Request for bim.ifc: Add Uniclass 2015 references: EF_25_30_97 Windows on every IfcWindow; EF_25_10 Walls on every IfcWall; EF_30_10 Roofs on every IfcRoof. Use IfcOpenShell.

First a look at what the model holds.

```python
import ifcopenshell

model = ifcopenshell.open("bim.ifc")
print(model.schema)
print("classifications:", [c.Name for c in model.by_type("IfcClassification")])
for ifc_class in ("IfcDoor", "IfcRoof", "IfcStair", "IfcWall", "IfcWindow"):
    print(ifc_class, len(model.by_type(ifc_class)))
```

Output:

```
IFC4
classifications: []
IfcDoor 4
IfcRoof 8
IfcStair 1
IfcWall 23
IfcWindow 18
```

```python
import ifcopenshell
import ifcopenshell.api.classification

model = ifcopenshell.open("bim.ifc")

system = ifcopenshell.api.classification.add_classification(model, classification="Uniclass 2015")

codes = {
    "IfcWindow": ("EF_25_30_97", "Windows"),
    "IfcWall": ("EF_25_10", "Walls"),
    "IfcRoof": ("EF_30_10", "Roofs"),
}
for ifc_class, (code, name) in codes.items():
    products = model.by_type(ifc_class)
    ifcopenshell.api.classification.add_reference(
        model, products=products, classification=system, identification=code, name=name
    )
    print(code, len(products))

model.write("bim_edited.ifc")
```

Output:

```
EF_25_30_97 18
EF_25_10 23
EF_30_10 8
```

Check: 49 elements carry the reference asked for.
